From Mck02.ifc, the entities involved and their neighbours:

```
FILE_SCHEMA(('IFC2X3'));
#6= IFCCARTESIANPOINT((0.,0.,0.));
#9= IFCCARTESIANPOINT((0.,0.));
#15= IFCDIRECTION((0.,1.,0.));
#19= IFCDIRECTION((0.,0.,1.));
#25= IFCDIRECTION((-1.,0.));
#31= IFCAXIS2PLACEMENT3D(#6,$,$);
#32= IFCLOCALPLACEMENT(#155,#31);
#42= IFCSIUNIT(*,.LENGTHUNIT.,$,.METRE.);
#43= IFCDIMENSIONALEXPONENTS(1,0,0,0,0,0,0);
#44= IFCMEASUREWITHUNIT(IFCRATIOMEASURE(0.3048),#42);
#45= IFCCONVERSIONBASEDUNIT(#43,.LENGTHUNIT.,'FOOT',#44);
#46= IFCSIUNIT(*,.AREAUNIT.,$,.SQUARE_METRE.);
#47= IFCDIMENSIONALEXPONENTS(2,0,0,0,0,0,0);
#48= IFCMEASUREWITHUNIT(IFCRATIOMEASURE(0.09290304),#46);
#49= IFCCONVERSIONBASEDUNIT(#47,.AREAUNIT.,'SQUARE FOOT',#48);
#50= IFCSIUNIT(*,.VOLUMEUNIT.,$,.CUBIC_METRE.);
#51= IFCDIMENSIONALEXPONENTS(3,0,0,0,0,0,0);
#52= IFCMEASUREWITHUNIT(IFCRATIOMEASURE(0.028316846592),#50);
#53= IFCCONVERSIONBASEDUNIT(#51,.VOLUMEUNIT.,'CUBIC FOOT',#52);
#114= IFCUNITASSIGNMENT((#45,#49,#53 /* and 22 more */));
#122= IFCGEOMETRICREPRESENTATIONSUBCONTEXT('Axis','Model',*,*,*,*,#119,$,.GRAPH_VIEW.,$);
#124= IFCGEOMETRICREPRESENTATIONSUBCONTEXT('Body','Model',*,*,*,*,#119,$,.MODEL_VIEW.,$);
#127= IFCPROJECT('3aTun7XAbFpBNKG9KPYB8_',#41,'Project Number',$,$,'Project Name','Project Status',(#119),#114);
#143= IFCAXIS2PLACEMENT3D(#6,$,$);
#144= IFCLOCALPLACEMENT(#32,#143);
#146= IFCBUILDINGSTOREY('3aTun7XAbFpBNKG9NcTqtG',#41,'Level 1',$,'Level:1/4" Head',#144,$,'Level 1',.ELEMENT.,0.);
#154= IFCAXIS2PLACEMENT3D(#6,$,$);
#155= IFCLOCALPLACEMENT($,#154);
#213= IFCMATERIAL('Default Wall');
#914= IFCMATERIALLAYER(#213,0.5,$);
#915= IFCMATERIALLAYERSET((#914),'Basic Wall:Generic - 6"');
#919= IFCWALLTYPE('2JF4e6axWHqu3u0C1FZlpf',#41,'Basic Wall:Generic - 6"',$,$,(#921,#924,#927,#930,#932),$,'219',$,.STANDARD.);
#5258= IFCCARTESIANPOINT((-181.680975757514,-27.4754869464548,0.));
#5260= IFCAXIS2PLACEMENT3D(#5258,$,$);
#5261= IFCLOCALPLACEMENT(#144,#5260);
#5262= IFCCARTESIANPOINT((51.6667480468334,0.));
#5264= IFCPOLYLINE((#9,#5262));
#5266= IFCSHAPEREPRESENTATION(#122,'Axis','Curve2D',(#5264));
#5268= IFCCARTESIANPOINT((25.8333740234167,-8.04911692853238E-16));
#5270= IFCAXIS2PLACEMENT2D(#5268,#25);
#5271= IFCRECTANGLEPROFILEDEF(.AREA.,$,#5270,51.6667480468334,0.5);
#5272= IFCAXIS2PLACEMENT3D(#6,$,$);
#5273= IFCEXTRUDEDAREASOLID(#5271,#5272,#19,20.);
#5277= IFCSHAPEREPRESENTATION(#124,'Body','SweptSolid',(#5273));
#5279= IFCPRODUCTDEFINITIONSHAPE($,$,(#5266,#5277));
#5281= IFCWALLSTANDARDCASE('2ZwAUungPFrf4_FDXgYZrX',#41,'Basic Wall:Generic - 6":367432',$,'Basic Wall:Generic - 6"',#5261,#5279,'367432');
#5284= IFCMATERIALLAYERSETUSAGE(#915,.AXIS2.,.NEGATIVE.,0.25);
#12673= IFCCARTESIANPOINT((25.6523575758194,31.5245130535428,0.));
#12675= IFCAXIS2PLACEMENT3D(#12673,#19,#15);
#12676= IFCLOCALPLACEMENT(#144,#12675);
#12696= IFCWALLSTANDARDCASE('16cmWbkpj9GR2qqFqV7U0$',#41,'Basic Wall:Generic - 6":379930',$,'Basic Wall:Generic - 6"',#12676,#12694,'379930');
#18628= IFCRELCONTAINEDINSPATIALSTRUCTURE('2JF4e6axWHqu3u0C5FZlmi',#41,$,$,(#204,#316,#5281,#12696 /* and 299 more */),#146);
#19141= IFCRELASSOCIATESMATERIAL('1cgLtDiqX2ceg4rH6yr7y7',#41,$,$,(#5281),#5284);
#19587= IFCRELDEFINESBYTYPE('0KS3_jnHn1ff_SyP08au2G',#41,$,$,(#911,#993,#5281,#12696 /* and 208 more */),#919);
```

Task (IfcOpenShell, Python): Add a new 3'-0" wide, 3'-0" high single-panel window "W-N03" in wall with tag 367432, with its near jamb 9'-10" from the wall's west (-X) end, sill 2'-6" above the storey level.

```python
import numpy as np
import ifcopenshell
import ifcopenshell.api.feature
import ifcopenshell.api.geometry
import ifcopenshell.api.root
import ifcopenshell.api.spatial
import ifcopenshell.api.type
import ifcopenshell.geom
import ifcopenshell.util.element
import ifcopenshell.util.placement
import ifcopenshell.util.representation
import ifcopenshell.util.shape
import ifcopenshell.util.unit

model = ifcopenshell.open("Mck02.ifc")
unit_scale = ifcopenshell.util.unit.calculate_unit_scale(model)
settings = ifcopenshell.geom.settings()


def volume(element):
    """Net volume in cubic metres, openings subtracted."""
    shape = ifcopenshell.geom.create_shape(settings, element)
    return ifcopenshell.util.shape.get_volume(shape.geometry)


wall = model.by_guid("2ZwAUungPFrf4_FDXgYZrX")
storey = ifcopenshell.util.element.get_container(wall, ifc_class="IfcBuildingStorey")
context = ifcopenshell.util.representation.get_context(model, "Model", "Body", "MODEL_VIEW")
before = volume(wall)

width, height, from_end, sill = 0.9144, 0.9144, 2.9972, 0.762  # metres

# The wall runs along its own X axis, and the end named is its -X end.
wall_shape = ifcopenshell.geom.create_shape(settings, wall)
x, y, z = ifcopenshell.util.shape.get_vertices(wall_shape.geometry).T
start = x.min() + from_end
face, thickness = float(y.min()), float(y.max() - y.min())
wall_matrix = ifcopenshell.util.placement.get_local_placement(wall.ObjectPlacement)
level = ifcopenshell.util.placement.get_local_placement(storey.ObjectPlacement)[2, 3]


def in_wall(x, y):
    """Placement at x, y metres in the wall's axes, at sill height."""
    matrix = wall_matrix.copy()
    matrix[:, 3] = wall_matrix @ np.array([x / unit_scale, y / unit_scale, 0.0, 1.0])
    matrix[2, 3] = level + sill / unit_scale
    return matrix


# Opening: a box that overshoots both wall faces by 50 mm.
opening = ifcopenshell.api.root.create_entity(model, ifc_class="IfcOpeningElement")
box = ifcopenshell.api.geometry.add_wall_representation(
    model, context=context, length=width, height=height, thickness=thickness + 0.1
)
ifcopenshell.api.geometry.assign_representation(model, product=opening, representation=box)
ifcopenshell.api.geometry.edit_object_placement(model, product=opening, matrix=in_wall(start, face - 0.05), is_si=False)
ifcopenshell.api.feature.add_feature(model, feature=opening, element=wall)

window = ifcopenshell.api.root.create_entity(model, ifc_class="IfcWindow", name="W-N03")
window.OverallWidth, window.OverallHeight = width / unit_scale, height / unit_scale
body = ifcopenshell.api.geometry.add_window_representation(
    model,
    context=context,
    overall_width=window.OverallWidth,
    overall_height=window.OverallHeight,
    partition_type="SINGLE_PANEL",
)
ifcopenshell.api.geometry.assign_representation(model, product=window, representation=body)
ifcopenshell.api.spatial.assign_container(model, products=[window], relating_structure=storey)
fills = ifcopenshell.api.feature.add_filling(model, opening=opening, element=window)
fills.OwnerHistory = window.OwnerHistory  # required in IFC2X3

# IFC2X3 keeps the operation on the window style.
style = ifcopenshell.api.root.create_entity(model, ifc_class="IfcWindowStyle", name="W-N03")
style.OperationType, style.ConstructionType = "SINGLE_PANEL", "NOTDEFINED"
style.ParameterTakesPrecedence = style.Sizeable = False
ifcopenshell.api.type.assign_type(model, related_objects=[window], relating_type=style)

# Centre the window in the wall's thickness.
ifcopenshell.api.geometry.edit_object_placement(model, product=window, matrix=in_wall(start, face), is_si=False)
window_shape = ifcopenshell.geom.create_shape(settings, window)
depth = ifcopenshell.util.shape.get_vertices(window_shape.geometry)[:, 1]
offset = face + thickness / 2 - (depth.min() + depth.max()) / 2
ifcopenshell.api.geometry.edit_object_placement(model, product=window, matrix=in_wall(start, offset), is_si=False)

after = volume(wall)

print(f"wall volume {before:.3f} -> {after:.3f} m3")

model.write("Mck02_v2.ifc")
```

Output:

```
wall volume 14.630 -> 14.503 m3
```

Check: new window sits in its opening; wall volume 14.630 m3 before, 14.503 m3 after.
